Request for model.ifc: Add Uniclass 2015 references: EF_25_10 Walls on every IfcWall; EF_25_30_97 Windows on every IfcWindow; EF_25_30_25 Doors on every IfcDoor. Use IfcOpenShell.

First a look at what the model holds.

```python
import ifcopenshell

model = ifcopenshell.open("model.ifc")
print(model.schema)
print("classifications:", [c.Name for c in model.by_type("IfcClassification")])
for ifc_class in ("IfcDoor", "IfcRoof", "IfcStair", "IfcWall", "IfcWindow"):
    print(ifc_class, len(model.by_type(ifc_class)))
```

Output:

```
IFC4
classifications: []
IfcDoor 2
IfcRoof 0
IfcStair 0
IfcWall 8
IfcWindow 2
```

```python
import ifcopenshell
import ifcopenshell.api.classification

model = ifcopenshell.open("model.ifc")

system = ifcopenshell.api.classification.add_classification(model, classification="Uniclass 2015")

codes = {
    "IfcWall": ("EF_25_10", "Walls"),
    "IfcWindow": ("EF_25_30_97", "Windows"),
    "IfcDoor": ("EF_25_30_25", "Doors"),
}
for ifc_class, (code, name) in codes.items():
    products = model.by_type(ifc_class)
    ifcopenshell.api.classification.add_reference(
        model, products=products, classification=system, identification=code, name=name
    )
    print(code, len(products))

model.write("model_edited.ifc")
```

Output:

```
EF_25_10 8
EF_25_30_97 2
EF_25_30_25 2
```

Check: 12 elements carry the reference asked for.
